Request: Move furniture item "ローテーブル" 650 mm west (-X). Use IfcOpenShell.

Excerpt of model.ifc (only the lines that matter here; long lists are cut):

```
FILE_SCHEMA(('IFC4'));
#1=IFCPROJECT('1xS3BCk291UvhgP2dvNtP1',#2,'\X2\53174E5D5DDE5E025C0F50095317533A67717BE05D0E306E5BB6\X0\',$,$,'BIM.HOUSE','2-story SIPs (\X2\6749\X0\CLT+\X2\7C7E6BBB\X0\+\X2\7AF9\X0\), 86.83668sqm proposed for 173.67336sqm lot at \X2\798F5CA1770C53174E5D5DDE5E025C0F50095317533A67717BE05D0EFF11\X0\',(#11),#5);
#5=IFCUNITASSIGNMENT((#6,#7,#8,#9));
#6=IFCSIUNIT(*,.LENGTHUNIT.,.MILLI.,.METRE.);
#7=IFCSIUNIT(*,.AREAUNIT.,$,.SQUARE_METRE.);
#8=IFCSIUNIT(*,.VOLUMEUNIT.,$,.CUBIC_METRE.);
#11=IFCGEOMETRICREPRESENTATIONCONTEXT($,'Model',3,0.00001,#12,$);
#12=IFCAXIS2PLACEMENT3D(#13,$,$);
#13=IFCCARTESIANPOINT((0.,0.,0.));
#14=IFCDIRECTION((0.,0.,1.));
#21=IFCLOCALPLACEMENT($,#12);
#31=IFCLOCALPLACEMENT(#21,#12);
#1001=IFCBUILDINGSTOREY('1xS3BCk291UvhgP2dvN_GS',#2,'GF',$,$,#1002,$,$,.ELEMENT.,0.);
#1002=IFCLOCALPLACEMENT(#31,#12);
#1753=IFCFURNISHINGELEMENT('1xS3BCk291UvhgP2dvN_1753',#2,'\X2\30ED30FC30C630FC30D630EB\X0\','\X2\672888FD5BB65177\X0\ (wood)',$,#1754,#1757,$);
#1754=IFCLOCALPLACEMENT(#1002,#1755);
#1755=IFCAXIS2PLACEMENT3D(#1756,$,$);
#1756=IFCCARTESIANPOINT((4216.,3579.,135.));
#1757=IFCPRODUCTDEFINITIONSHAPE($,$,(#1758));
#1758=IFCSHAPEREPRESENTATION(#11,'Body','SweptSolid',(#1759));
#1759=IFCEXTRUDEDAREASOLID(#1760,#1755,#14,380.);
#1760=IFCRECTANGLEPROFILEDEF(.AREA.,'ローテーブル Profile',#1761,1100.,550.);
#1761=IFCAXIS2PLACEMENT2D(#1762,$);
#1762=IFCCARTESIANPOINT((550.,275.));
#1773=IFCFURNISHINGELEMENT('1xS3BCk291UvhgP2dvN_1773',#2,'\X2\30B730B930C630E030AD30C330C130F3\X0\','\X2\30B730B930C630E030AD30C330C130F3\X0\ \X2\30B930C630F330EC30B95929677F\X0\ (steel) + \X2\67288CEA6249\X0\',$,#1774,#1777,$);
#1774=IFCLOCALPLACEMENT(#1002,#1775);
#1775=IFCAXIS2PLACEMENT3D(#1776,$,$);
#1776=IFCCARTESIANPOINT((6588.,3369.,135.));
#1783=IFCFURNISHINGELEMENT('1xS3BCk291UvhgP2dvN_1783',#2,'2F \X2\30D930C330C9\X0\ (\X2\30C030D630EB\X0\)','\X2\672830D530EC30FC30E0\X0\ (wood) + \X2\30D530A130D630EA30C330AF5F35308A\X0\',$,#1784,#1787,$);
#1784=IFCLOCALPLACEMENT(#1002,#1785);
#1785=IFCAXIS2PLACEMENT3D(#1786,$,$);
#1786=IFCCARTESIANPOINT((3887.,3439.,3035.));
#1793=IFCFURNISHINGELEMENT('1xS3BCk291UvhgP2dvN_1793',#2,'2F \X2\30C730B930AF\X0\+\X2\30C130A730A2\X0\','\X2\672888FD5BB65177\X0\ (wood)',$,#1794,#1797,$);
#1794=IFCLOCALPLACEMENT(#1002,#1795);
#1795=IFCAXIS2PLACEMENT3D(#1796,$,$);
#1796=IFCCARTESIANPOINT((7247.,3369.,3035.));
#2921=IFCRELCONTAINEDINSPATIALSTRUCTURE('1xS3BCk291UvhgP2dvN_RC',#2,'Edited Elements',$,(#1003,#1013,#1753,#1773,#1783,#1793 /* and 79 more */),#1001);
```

```python
import ifcopenshell
import ifcopenshell.api.geometry
import ifcopenshell.util.placement
import ifcopenshell.util.unit

model = ifcopenshell.open("model.ifc")
unit_scale = ifcopenshell.util.unit.calculate_unit_scale(model)

item = model.by_guid("1xS3BCk291UvhgP2dvN_1753")
matrix = ifcopenshell.util.placement.get_local_placement(item.ObjectPlacement)
matrix[0, 3] -= 0.65 / unit_scale
ifcopenshell.api.geometry.edit_object_placement(model, product=item, matrix=matrix, is_si=False)

print(ifcopenshell.util.placement.get_local_placement(item.ObjectPlacement).round(3) + 0.0)

model.write("model_v2.ifc")
```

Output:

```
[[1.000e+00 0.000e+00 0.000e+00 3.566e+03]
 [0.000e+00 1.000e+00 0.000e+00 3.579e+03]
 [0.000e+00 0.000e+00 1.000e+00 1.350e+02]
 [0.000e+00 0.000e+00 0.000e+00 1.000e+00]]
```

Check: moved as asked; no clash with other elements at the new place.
